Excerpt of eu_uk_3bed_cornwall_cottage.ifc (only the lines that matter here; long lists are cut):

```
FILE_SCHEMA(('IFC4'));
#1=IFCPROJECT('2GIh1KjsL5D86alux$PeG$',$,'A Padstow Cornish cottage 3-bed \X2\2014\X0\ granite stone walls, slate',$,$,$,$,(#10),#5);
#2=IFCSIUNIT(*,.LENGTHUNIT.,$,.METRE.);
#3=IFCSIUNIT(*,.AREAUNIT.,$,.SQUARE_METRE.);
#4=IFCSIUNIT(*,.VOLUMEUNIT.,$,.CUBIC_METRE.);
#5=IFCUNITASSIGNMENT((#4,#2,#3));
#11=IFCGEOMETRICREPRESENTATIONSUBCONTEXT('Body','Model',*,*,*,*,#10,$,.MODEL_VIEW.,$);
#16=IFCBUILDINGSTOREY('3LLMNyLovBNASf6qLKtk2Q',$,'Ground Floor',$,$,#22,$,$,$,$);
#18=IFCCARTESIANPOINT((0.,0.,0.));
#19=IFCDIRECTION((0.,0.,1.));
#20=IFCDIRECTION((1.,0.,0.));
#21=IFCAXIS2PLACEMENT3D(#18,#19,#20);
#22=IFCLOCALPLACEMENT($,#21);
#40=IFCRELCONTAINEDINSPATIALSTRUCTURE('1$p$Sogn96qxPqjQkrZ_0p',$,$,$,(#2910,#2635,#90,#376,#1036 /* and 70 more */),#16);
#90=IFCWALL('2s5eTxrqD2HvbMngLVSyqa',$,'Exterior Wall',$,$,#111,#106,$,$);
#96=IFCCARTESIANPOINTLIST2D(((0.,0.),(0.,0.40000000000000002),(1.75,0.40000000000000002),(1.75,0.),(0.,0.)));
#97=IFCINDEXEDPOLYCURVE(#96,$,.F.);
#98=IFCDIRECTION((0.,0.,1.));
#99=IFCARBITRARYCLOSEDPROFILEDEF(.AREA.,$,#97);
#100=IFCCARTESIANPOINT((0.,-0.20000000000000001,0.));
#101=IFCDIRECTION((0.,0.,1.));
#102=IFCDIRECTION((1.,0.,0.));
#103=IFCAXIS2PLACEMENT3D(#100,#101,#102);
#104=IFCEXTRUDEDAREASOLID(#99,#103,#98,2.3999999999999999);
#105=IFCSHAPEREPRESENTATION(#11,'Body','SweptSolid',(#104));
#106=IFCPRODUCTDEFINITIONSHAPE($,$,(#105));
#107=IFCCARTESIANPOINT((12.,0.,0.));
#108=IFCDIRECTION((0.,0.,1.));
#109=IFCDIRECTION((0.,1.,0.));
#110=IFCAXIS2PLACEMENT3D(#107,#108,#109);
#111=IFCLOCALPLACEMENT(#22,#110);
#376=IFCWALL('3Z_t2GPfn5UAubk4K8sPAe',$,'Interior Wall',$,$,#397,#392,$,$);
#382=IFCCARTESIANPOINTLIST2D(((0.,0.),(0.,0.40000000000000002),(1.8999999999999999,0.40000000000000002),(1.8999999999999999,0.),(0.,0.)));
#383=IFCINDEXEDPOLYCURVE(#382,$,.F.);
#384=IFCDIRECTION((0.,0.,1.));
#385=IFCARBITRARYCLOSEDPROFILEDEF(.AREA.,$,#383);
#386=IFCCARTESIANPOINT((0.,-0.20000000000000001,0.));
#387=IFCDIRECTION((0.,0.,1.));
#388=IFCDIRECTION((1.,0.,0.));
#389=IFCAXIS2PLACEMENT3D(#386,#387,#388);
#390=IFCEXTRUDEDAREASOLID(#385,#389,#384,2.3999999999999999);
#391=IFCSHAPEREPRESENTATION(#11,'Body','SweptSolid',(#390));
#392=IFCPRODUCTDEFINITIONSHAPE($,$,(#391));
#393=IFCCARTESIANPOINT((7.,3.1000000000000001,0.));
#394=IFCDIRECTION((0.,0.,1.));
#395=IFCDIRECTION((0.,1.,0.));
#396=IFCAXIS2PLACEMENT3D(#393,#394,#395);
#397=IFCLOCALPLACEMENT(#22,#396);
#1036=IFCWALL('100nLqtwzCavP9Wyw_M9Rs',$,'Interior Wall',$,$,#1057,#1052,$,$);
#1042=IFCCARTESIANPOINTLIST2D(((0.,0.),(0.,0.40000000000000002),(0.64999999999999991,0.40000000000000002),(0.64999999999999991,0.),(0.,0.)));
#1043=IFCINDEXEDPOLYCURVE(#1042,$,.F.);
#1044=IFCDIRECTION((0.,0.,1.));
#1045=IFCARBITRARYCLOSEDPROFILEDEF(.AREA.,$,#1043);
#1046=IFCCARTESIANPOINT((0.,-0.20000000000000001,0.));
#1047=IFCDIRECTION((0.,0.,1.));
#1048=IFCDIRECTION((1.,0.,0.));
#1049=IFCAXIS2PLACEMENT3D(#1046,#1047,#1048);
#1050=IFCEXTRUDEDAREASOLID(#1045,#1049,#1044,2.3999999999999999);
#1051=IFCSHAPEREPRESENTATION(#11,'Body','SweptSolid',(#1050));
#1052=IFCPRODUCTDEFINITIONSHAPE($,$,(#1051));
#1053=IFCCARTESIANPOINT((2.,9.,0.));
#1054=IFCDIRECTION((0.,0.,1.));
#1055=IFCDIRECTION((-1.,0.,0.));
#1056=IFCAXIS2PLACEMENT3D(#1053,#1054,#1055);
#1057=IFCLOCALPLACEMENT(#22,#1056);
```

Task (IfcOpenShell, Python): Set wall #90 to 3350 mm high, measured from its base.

```python
import ifcopenshell
import ifcopenshell.geom
import ifcopenshell.util.representation
import ifcopenshell.util.shape
import ifcopenshell.util.unit

model = ifcopenshell.open("eu_uk_3bed_cornwall_cottage.ifc")
unit_scale = ifcopenshell.util.unit.calculate_unit_scale(model)
settings = ifcopenshell.geom.settings()


def volume(element):
    """Net volume in cubic metres, openings subtracted."""
    shape = ifcopenshell.geom.create_shape(settings, element)
    return ifcopenshell.util.shape.get_volume(shape.geometry)


wall = model.by_guid("2s5eTxrqD2HvbMngLVSyqa")
before = volume(wall)

body = ifcopenshell.util.representation.get_representation(wall, "Model", "Body")
solid = body.Items[0]
old_height = solid.Depth
solid.Depth = 3.35 / unit_scale
after = volume(wall)

print(f"height {old_height:g} -> {solid.Depth:g}, volume {before:.3f} -> {after:.3f} m3")

model.write("eu_uk_3bed_cornwall_cottage_edited.ifc")
```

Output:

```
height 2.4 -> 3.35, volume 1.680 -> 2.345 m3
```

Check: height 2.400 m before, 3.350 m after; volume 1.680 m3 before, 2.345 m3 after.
